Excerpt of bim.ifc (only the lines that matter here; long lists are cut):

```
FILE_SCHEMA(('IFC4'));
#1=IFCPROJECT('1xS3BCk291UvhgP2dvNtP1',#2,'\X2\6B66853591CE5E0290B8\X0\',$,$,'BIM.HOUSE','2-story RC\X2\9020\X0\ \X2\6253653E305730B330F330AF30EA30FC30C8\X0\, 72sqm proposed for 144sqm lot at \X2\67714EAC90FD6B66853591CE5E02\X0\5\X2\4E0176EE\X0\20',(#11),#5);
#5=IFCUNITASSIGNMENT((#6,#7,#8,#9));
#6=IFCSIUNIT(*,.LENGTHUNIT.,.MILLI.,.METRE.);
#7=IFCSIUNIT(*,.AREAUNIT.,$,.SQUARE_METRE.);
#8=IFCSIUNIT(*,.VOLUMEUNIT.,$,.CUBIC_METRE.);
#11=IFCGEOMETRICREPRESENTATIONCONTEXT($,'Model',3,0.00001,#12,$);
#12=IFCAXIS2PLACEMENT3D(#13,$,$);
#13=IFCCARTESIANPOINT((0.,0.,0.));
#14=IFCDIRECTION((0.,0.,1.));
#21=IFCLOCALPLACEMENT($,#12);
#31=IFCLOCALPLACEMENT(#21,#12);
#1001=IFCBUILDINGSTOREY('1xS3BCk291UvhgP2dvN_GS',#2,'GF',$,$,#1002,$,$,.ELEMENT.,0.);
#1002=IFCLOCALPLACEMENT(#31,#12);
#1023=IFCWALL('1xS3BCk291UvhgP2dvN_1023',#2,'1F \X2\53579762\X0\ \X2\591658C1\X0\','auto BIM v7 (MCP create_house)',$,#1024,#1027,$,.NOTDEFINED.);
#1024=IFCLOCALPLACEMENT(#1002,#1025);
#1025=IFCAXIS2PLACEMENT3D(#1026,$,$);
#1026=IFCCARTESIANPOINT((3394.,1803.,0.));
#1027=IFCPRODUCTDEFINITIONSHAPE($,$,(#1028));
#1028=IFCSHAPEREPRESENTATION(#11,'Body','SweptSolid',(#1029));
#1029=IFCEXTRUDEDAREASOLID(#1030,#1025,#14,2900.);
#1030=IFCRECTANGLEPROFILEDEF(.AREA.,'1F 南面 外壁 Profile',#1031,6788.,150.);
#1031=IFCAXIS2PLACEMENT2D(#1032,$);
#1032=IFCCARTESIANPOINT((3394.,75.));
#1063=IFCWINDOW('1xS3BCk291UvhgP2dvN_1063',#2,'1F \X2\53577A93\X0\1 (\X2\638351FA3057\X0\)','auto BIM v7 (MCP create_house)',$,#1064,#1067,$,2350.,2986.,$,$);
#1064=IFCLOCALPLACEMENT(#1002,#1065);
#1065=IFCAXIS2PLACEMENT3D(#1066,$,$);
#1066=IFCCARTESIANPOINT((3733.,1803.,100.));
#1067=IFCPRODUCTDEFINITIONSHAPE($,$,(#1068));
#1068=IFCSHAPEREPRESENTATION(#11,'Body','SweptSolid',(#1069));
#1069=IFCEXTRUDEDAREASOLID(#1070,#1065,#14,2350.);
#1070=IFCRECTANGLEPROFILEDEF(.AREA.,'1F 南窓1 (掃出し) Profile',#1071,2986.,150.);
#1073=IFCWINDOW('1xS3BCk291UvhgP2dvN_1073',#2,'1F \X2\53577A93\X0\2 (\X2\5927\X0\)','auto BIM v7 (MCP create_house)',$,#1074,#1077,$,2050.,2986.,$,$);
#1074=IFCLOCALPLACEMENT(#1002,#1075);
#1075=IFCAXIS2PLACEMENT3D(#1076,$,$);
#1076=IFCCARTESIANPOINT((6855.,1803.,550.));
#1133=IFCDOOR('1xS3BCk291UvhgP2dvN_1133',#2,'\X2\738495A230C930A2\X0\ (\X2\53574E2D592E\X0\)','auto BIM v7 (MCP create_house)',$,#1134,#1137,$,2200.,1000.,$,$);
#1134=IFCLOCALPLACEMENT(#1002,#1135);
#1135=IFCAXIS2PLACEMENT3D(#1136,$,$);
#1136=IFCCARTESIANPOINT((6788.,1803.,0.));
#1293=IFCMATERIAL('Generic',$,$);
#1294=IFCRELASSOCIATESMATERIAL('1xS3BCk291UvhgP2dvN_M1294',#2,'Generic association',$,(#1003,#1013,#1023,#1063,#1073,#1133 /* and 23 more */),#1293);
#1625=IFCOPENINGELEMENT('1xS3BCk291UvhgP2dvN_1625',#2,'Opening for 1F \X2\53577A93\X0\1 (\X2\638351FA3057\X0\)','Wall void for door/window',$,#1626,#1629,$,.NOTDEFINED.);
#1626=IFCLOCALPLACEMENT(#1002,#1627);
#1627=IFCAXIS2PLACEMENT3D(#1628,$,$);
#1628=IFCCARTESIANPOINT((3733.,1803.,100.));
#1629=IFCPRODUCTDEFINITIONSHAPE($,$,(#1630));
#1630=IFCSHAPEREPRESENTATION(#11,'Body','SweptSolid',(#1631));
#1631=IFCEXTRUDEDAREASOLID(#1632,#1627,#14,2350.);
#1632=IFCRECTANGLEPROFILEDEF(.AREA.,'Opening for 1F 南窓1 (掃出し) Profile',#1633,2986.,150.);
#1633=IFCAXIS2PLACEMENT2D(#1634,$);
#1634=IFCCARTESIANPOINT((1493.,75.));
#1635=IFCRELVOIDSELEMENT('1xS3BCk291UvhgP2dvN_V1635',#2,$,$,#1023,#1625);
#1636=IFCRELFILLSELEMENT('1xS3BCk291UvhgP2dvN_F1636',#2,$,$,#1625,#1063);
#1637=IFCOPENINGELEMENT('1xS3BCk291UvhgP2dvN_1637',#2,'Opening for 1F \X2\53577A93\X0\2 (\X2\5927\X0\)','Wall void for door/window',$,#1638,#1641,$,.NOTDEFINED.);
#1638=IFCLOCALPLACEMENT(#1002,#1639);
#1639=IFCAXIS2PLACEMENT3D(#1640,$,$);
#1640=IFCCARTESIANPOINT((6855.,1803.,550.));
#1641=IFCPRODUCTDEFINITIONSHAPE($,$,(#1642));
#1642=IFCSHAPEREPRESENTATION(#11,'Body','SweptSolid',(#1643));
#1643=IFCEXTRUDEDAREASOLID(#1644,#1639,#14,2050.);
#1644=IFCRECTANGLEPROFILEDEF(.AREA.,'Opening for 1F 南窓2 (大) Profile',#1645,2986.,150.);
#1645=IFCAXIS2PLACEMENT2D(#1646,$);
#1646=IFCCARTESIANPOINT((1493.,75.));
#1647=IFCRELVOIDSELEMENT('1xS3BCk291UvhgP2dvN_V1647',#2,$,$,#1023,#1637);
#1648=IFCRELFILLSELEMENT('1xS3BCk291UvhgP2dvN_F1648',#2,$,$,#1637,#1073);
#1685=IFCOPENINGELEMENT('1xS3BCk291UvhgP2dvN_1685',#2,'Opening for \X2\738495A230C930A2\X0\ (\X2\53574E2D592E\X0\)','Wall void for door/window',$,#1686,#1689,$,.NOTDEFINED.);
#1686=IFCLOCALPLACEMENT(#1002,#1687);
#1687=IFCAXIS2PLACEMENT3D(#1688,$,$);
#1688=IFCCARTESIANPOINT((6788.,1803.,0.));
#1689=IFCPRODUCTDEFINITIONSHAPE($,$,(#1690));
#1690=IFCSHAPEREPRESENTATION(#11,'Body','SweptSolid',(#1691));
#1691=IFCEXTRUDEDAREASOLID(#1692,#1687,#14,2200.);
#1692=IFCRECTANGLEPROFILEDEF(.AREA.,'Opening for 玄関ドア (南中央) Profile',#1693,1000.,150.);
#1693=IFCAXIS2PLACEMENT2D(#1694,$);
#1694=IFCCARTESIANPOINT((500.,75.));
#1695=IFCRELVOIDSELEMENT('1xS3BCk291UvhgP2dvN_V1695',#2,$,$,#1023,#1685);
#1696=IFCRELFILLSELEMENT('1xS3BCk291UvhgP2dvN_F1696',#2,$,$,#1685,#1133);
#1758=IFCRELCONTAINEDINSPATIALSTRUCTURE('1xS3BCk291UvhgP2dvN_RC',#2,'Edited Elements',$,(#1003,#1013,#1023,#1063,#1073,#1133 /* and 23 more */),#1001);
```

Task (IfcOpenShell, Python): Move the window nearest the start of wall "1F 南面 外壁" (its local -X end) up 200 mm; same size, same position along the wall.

```python
import numpy as np
import ifcopenshell
import ifcopenshell.api.geometry
import ifcopenshell.util.placement
import ifcopenshell.util.unit

model = ifcopenshell.open("bim.ifc")
unit_scale = ifcopenshell.util.unit.calculate_unit_scale(model)

window = model.by_guid("1xS3BCk291UvhgP2dvN_1063")
opening = window.FillsVoids[0].RelatingOpeningElement
dz = 200.0

shift = np.array([0.0, 0.0, dz])
# The window is not placed relative to its opening, so move both.
for product in (opening, window):
    matrix = ifcopenshell.util.placement.get_local_placement(product.ObjectPlacement)
    matrix[:3, 3] += shift
    ifcopenshell.api.geometry.edit_object_placement(model, product=product, matrix=matrix, is_si=False)

print(f"moved by {dz * unit_scale:+.3f} m")

model.write("bim_v2.ifc")
```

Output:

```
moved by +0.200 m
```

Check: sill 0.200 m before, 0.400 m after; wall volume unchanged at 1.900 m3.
